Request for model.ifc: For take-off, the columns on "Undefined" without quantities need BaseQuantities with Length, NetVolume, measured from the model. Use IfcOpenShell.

First a look at what the model holds.

```python
import ifcopenshell
import ifcopenshell.util.element
import ifcopenshell.util.unit

model = ifcopenshell.open("model.ifc")
print(model.schema)
for unit_type in ("LENGTHUNIT", "AREAUNIT", "VOLUMEUNIT"):
    print(unit_type, ifcopenshell.util.unit.calculate_unit_scale(model, unit_type))
storey = next(s for s in model.by_type("IfcBuildingStorey") if s.Name == "Undefined")
columns = [e for e in ifcopenshell.util.element.get_decomposition(storey) if e.is_a("IfcColumn")]
for e in sorted(columns, key=lambda e: e.id()):
    print(e.id(), e.is_a(), e.Name, list(ifcopenshell.util.element.get_psets(e, qtos_only=True)), sep=" | ")
```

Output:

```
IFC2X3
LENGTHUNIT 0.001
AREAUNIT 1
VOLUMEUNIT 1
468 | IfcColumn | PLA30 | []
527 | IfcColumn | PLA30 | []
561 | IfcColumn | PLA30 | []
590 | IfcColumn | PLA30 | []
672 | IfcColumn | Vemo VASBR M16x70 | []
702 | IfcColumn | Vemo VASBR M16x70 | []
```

```python
import ifcopenshell
import ifcopenshell.api.pset
import ifcopenshell.geom
import ifcopenshell.util.element
import ifcopenshell.util.shape
import ifcopenshell.util.unit

model = ifcopenshell.open("model.ifc")
unit_scale = ifcopenshell.util.unit.calculate_unit_scale(model)
volume_scale = ifcopenshell.util.unit.calculate_unit_scale(model, "VOLUMEUNIT")
settings = ifcopenshell.geom.settings()

storey = next(s for s in model.by_type("IfcBuildingStorey") if s.Name == "Undefined")
columns = [e for e in ifcopenshell.util.element.get_decomposition(storey) if e.is_a("IfcColumn")]

for e in sorted(columns, key=lambda e: e.id()):
    if ifcopenshell.util.element.get_psets(e, qtos_only=True, should_inherit=False):
        continue
    # Geometry comes back in metres, in the element's own axes.
    shape = ifcopenshell.geom.create_shape(settings, e)
    values = {
        "Length": ifcopenshell.util.shape.get_z(shape.geometry) / unit_scale,
        "NetVolume": ifcopenshell.util.shape.get_volume(shape.geometry) / volume_scale,
    }
    qto = ifcopenshell.api.pset.add_qto(model, product=e, name="BaseQuantities")
    ifcopenshell.api.pset.edit_qto(model, qto=qto, properties=values)
    print(e.id(), {k: round(v, 3) for k, v in values.items()})

model.write("model_updated.ifc")
```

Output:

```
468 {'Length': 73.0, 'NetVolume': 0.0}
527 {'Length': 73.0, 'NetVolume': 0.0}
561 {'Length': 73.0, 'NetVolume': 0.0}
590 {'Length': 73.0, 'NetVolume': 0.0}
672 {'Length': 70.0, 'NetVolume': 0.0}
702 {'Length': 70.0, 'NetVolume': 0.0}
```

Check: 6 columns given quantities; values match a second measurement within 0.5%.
